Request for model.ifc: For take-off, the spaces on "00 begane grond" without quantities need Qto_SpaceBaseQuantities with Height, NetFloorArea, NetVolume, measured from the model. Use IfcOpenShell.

First a look at what the model holds.

```python
import ifcopenshell
import ifcopenshell.util.element
import ifcopenshell.util.unit

model = ifcopenshell.open("model.ifc")
print(model.schema)
for unit_type in ("LENGTHUNIT", "AREAUNIT", "VOLUMEUNIT"):
    print(unit_type, ifcopenshell.util.unit.calculate_unit_scale(model, unit_type))
storey = next(s for s in model.by_type("IfcBuildingStorey") if s.Name == "00 begane grond")
spaces = [e for e in ifcopenshell.util.element.get_decomposition(storey) if e.is_a("IfcSpace")]
for e in sorted(spaces, key=lambda e: e.id()):
    print(e.id(), e.is_a(), e.Name, list(ifcopenshell.util.element.get_psets(e, qtos_only=True)), sep=" | ")
```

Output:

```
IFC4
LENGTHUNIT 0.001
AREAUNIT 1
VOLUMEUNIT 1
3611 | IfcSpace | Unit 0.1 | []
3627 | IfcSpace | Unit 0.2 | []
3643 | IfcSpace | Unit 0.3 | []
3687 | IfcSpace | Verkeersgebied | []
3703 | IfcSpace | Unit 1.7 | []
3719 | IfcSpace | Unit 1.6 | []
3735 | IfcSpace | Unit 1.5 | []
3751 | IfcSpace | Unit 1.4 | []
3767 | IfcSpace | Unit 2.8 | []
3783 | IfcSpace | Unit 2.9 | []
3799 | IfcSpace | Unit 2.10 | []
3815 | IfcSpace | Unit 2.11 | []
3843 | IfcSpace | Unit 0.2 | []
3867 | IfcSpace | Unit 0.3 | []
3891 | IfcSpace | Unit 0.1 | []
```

```python
import ifcopenshell
import ifcopenshell.api.pset
import ifcopenshell.geom
import ifcopenshell.util.element
import ifcopenshell.util.shape
import ifcopenshell.util.unit

model = ifcopenshell.open("model.ifc")
unit_scale = ifcopenshell.util.unit.calculate_unit_scale(model)
area_scale = ifcopenshell.util.unit.calculate_unit_scale(model, "AREAUNIT")
volume_scale = ifcopenshell.util.unit.calculate_unit_scale(model, "VOLUMEUNIT")
settings = ifcopenshell.geom.settings()

storey = next(s for s in model.by_type("IfcBuildingStorey") if s.Name == "00 begane grond")
spaces = [e for e in ifcopenshell.util.element.get_decomposition(storey) if e.is_a("IfcSpace")]

for e in sorted(spaces, key=lambda e: e.id()):
    if ifcopenshell.util.element.get_psets(e, qtos_only=True, should_inherit=False):
        continue
    # Geometry comes back in metres, in the element's own axes.
    shape = ifcopenshell.geom.create_shape(settings, e)
    values = {
        "Height": ifcopenshell.util.shape.get_z(shape.geometry) / unit_scale,
        "NetFloorArea": ifcopenshell.util.shape.get_footprint_area(shape.geometry) / area_scale,
        "NetVolume": ifcopenshell.util.shape.get_volume(shape.geometry) / volume_scale,
    }
    qto = ifcopenshell.api.pset.add_qto(model, product=e, name="Qto_SpaceBaseQuantities")
    ifcopenshell.api.pset.edit_qto(model, qto=qto, properties=values)
    print(e.id(), {k: round(v, 3) for k, v in values.items()})

model.write("model_rev.ifc")
```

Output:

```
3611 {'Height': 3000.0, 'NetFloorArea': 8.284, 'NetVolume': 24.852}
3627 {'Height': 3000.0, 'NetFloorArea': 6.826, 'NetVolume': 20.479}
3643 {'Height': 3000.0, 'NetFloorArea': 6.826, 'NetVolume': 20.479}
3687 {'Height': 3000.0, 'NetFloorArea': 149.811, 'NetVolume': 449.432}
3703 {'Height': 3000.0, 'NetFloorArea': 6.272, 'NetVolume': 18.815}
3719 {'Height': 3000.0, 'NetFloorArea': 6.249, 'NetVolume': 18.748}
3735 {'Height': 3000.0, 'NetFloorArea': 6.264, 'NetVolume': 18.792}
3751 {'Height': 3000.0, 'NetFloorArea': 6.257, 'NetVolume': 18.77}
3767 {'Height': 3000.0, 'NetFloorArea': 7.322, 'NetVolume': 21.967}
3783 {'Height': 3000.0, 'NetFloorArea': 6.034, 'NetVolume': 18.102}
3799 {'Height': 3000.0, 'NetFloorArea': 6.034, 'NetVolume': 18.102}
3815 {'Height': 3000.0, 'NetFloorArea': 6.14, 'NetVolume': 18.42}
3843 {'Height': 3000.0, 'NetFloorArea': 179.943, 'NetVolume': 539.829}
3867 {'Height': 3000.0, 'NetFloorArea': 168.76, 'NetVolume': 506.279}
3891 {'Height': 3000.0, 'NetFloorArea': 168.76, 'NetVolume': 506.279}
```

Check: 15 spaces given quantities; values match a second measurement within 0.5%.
